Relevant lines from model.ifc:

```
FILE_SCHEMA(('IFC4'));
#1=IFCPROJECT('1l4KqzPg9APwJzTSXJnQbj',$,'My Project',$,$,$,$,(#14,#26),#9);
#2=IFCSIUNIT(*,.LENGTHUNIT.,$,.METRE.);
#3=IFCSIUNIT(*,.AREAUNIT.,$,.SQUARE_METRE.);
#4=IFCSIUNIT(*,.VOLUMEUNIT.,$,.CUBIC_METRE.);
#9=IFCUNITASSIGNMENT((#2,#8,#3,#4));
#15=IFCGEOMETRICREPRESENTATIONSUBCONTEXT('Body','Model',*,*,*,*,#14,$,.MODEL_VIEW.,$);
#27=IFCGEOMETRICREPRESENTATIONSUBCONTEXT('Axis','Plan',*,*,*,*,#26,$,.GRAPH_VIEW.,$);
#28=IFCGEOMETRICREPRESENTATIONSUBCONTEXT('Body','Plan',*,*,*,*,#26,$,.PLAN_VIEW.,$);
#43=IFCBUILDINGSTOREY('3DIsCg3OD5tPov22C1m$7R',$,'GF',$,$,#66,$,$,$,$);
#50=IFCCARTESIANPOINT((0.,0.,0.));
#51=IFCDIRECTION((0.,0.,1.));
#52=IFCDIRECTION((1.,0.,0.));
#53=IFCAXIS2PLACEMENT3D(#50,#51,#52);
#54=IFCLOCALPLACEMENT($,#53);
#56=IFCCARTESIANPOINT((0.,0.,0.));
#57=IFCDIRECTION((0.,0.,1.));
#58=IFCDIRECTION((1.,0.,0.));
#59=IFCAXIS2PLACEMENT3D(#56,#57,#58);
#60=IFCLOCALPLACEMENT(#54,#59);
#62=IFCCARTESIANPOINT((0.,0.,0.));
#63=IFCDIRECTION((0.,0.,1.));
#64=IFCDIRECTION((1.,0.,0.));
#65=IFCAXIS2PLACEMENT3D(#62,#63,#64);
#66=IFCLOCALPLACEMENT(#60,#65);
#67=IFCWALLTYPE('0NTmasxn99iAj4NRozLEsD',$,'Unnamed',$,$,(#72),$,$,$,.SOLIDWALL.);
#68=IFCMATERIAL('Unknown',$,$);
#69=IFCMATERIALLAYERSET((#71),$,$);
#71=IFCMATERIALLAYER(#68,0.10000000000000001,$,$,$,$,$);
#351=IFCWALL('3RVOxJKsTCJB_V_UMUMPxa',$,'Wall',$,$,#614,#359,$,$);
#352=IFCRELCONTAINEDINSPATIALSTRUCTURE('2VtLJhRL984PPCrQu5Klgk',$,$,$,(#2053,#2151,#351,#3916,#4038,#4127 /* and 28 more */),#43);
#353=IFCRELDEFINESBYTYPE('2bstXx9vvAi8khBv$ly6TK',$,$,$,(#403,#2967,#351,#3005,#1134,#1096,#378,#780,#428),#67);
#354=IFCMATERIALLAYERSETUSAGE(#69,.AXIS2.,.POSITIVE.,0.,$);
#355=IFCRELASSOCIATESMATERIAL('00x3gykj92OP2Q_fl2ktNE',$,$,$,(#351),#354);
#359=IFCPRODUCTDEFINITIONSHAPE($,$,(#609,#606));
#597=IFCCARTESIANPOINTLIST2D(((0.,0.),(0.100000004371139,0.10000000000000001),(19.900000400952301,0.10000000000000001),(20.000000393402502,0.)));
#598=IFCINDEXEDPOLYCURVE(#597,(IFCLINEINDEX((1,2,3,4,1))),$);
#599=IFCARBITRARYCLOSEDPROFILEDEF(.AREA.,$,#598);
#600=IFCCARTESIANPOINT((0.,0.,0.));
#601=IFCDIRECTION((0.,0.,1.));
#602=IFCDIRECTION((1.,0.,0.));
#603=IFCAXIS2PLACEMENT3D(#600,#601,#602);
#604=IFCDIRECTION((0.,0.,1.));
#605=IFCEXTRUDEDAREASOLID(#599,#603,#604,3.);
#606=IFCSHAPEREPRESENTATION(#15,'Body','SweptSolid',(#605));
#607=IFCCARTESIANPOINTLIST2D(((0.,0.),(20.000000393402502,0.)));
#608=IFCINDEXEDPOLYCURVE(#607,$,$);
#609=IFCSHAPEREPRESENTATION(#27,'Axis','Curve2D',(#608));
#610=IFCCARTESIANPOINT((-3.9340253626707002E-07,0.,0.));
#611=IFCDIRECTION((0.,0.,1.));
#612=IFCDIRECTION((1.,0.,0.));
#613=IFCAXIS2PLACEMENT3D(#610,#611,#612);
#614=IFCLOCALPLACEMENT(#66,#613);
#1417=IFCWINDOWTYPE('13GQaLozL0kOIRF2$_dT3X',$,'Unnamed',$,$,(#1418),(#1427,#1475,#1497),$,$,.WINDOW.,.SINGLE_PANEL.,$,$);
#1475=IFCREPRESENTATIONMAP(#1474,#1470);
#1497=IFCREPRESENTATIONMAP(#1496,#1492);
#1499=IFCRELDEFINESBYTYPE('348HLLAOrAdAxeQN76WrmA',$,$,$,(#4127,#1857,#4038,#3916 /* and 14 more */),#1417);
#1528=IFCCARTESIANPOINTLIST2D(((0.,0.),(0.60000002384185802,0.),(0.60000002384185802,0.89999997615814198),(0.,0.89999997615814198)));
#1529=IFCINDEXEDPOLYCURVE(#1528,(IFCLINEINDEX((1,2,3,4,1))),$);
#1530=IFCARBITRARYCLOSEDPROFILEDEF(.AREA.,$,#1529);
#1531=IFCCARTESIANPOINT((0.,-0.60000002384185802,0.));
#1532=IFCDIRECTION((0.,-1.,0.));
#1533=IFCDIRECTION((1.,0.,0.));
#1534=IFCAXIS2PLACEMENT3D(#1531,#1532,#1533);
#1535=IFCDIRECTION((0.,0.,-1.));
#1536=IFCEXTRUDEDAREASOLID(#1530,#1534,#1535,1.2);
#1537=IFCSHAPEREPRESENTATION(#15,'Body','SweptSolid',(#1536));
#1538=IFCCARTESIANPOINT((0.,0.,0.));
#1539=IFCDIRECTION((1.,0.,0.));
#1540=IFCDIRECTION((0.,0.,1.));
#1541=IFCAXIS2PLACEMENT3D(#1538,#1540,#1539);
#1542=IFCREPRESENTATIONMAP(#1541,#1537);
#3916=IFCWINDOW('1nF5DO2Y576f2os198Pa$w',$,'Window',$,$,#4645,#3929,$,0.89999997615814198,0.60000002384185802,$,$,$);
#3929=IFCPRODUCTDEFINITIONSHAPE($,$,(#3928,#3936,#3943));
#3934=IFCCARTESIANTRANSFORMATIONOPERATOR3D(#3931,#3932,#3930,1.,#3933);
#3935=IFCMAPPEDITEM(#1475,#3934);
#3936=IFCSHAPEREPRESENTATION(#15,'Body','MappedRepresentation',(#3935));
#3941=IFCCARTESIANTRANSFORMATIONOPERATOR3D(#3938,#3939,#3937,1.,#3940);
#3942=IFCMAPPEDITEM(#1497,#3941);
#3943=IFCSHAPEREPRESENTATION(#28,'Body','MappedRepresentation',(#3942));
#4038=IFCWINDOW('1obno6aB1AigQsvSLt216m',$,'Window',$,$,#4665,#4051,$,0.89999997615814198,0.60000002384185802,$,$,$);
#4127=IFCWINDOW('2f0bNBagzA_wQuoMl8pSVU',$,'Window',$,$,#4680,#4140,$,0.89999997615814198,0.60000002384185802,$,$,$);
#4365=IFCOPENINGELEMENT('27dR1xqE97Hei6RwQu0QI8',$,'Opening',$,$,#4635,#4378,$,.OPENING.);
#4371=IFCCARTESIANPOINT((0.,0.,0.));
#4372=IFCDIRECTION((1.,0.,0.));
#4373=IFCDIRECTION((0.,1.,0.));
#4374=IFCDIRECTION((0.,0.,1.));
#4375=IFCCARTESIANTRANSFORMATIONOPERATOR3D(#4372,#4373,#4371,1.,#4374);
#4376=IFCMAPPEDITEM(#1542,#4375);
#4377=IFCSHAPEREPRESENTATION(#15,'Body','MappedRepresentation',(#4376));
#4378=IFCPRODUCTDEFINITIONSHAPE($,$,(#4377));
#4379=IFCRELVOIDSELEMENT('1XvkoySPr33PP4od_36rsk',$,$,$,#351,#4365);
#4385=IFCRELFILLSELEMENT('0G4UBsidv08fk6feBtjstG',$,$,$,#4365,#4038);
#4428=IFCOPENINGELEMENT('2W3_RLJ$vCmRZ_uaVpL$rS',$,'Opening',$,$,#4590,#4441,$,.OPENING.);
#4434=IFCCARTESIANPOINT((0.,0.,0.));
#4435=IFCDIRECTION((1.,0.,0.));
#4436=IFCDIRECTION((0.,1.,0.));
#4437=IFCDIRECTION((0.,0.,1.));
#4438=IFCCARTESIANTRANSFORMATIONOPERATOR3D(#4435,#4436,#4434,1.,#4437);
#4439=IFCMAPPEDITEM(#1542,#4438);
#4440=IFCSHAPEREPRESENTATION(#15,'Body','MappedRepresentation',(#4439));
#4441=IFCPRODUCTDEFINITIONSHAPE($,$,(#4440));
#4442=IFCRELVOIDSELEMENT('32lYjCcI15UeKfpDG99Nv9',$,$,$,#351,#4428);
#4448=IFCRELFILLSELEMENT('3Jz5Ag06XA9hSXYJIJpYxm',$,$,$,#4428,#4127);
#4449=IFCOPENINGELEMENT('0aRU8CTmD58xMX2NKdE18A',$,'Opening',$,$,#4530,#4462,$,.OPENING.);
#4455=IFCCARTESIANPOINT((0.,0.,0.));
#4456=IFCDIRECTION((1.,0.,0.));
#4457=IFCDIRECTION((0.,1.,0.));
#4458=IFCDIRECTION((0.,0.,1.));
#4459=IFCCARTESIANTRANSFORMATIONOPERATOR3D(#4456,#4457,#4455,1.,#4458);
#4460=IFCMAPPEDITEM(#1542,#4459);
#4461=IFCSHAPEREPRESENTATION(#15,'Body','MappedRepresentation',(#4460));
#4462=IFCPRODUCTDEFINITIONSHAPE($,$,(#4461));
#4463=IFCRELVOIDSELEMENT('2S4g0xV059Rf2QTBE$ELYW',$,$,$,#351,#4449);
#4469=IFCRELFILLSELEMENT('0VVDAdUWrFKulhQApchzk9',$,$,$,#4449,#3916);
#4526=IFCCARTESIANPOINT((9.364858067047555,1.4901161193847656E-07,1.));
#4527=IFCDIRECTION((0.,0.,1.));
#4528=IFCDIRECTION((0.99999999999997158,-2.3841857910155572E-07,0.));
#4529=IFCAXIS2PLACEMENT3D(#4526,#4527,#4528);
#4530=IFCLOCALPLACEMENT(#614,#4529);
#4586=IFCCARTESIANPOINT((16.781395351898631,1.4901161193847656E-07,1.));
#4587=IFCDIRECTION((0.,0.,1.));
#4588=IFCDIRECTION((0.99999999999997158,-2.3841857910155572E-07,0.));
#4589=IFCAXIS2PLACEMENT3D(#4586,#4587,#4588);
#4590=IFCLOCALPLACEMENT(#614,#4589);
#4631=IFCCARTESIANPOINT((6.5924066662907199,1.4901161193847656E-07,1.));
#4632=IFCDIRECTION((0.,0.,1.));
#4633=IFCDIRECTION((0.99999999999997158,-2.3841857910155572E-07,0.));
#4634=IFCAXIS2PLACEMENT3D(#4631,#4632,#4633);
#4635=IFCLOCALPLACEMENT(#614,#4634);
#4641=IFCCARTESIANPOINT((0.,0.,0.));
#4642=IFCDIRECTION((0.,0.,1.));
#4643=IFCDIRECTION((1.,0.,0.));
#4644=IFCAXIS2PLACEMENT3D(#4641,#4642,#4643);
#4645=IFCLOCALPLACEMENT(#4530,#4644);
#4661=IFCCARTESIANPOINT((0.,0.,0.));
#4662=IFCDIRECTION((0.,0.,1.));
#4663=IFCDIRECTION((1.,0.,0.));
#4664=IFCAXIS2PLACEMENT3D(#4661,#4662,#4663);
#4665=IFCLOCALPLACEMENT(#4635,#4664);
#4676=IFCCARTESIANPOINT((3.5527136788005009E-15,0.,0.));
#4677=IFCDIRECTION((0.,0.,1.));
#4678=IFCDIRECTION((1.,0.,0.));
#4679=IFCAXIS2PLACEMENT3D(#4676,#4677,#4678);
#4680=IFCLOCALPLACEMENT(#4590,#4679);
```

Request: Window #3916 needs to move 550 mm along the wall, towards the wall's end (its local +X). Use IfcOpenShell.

```python
import ifcopenshell
import ifcopenshell.api.geometry
import ifcopenshell.util.placement
import ifcopenshell.util.unit

model = ifcopenshell.open("model.ifc")
unit_scale = ifcopenshell.util.unit.calculate_unit_scale(model)

window = model.by_id(3916)
opening = window.FillsVoids[0].RelatingOpeningElement
wall = opening.VoidsElements[0].RelatingBuildingElement

wall_matrix = ifcopenshell.util.placement.get_local_placement(wall.ObjectPlacement)
shift = wall_matrix[:3, 0] * 0.55 / unit_scale
before = ifcopenshell.util.placement.get_local_placement(window.ObjectPlacement)[:3, 3].copy()

# The window is placed relative to its opening, so it follows when the opening moves.
matrix = ifcopenshell.util.placement.get_local_placement(opening.ObjectPlacement)
matrix[:3, 3] += shift
ifcopenshell.api.geometry.edit_object_placement(
    model, product=opening, matrix=matrix, is_si=False, should_transform_children=True
)

after = ifcopenshell.util.placement.get_local_placement(window.ObjectPlacement)[:3, 3]
print("window moved by", (after - before).round(3) + 0.0)

model.write("model-out.ifc")
```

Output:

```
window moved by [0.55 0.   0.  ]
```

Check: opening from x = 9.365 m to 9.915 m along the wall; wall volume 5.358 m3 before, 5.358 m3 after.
